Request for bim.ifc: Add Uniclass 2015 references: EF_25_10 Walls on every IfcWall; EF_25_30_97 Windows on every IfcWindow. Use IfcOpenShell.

First a look at what the model holds.

```python
import ifcopenshell

model = ifcopenshell.open("bim.ifc")
print(model.schema)
print("classifications:", [c.Name for c in model.by_type("IfcClassification")])
for ifc_class in ("IfcDoor", "IfcRoof", "IfcStair", "IfcWall", "IfcWindow"):
    print(ifc_class, len(model.by_type(ifc_class)))
```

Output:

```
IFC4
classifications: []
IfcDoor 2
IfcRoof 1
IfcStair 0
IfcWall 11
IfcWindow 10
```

```python
import ifcopenshell
import ifcopenshell.api.classification

model = ifcopenshell.open("bim.ifc")

system = ifcopenshell.api.classification.add_classification(model, classification="Uniclass 2015")

codes = {
    "IfcWall": ("EF_25_10", "Walls"),
    "IfcWindow": ("EF_25_30_97", "Windows"),
}
for ifc_class, (code, name) in codes.items():
    products = model.by_type(ifc_class)
    ifcopenshell.api.classification.add_reference(
        model, products=products, classification=system, identification=code, name=name
    )
    print(code, len(products))

model.write("bim_rev.ifc")
```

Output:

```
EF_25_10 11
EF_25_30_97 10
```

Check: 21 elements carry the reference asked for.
